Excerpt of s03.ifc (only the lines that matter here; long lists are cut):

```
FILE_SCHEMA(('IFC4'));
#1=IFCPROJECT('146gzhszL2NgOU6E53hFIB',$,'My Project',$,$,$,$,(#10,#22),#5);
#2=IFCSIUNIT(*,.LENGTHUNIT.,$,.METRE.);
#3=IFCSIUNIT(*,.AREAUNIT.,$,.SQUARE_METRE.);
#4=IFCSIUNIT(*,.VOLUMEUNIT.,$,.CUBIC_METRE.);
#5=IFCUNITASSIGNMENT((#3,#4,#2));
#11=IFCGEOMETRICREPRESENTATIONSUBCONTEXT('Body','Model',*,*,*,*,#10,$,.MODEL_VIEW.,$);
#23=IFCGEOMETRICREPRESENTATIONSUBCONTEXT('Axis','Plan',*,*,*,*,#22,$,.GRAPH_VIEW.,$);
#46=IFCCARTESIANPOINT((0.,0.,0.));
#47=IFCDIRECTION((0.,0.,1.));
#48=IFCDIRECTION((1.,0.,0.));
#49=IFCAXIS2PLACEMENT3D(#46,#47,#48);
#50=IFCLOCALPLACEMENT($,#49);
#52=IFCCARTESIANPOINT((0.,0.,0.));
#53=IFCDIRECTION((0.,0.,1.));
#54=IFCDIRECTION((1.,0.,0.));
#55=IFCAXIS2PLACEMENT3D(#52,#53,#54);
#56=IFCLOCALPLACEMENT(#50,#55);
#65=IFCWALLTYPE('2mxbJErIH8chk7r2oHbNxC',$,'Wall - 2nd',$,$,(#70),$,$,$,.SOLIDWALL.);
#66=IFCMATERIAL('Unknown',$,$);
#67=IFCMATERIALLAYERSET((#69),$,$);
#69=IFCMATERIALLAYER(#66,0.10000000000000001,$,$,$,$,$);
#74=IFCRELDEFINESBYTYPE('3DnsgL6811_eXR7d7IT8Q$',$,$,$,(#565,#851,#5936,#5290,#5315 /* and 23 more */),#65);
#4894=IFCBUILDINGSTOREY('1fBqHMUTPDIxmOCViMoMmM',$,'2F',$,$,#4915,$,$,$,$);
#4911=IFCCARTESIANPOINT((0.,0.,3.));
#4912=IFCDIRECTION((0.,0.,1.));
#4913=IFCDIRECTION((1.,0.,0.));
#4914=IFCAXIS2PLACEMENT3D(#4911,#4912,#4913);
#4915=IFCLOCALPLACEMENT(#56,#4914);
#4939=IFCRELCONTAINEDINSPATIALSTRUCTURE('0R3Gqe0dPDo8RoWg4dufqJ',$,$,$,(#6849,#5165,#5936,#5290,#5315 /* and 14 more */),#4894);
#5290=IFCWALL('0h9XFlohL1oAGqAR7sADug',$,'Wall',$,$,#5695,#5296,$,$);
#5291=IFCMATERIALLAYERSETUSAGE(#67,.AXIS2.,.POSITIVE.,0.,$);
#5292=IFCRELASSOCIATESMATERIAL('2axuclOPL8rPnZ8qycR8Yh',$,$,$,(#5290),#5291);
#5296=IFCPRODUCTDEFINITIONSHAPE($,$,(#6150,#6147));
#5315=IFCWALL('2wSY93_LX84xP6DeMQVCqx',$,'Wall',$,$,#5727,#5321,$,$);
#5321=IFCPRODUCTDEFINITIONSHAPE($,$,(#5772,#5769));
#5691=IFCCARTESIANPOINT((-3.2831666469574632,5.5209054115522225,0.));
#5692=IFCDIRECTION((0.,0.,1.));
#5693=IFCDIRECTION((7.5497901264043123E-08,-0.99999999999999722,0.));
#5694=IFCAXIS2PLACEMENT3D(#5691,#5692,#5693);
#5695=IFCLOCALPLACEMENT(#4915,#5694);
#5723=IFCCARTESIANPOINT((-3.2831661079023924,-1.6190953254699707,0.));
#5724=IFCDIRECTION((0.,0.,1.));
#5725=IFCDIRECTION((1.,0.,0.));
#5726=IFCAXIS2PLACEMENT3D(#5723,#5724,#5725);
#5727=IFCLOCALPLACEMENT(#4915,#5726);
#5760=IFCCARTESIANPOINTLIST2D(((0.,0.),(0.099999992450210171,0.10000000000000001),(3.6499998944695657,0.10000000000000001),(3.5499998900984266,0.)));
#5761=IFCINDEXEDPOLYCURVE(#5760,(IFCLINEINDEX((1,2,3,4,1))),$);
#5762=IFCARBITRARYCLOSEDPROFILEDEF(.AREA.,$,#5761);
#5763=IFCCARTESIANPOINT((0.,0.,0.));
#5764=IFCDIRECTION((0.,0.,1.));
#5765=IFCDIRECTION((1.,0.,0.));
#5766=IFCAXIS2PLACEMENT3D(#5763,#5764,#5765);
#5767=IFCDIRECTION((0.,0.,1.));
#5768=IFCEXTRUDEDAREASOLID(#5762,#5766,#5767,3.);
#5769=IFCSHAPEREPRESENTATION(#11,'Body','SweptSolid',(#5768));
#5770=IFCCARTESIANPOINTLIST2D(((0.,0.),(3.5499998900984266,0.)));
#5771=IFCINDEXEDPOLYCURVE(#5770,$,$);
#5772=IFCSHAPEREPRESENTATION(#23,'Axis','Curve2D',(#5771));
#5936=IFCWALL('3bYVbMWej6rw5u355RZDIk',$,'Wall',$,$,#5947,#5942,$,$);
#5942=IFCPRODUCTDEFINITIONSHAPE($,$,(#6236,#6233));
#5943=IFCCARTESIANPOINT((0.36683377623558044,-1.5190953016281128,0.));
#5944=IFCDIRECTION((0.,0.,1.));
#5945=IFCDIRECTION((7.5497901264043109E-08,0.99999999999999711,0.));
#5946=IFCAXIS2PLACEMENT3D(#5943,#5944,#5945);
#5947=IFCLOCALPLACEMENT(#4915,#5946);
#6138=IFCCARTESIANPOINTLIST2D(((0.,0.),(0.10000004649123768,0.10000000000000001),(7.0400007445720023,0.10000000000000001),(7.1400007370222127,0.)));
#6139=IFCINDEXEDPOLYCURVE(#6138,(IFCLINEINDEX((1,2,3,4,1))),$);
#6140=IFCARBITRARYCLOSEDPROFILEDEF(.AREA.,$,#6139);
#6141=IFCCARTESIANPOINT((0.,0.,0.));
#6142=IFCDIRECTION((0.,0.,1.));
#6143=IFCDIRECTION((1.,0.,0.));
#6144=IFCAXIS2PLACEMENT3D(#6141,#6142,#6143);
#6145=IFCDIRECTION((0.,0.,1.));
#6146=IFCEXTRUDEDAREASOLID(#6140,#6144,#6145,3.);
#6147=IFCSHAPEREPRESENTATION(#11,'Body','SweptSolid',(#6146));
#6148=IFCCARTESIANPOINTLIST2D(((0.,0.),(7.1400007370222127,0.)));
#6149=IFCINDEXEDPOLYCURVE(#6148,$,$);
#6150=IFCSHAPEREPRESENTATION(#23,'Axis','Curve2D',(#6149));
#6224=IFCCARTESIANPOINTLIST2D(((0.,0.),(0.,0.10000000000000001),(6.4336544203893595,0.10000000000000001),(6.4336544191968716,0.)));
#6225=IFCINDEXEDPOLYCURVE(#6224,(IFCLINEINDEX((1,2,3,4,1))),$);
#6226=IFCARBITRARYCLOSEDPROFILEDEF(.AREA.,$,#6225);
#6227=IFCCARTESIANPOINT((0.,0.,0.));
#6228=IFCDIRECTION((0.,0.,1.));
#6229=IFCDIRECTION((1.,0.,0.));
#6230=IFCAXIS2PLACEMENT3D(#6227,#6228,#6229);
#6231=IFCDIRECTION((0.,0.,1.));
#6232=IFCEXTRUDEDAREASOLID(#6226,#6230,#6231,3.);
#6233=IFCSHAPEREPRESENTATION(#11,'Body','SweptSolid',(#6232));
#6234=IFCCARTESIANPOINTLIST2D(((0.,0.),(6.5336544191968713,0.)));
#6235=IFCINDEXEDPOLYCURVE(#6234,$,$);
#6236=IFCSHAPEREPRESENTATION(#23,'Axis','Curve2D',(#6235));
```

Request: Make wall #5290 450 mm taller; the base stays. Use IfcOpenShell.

```python
import ifcopenshell
import ifcopenshell.geom
import ifcopenshell.util.representation
import ifcopenshell.util.shape
import ifcopenshell.util.unit

model = ifcopenshell.open("s03.ifc")
unit_scale = ifcopenshell.util.unit.calculate_unit_scale(model)
settings = ifcopenshell.geom.settings()


def volume(element):
    """Net volume in cubic metres, openings subtracted."""
    shape = ifcopenshell.geom.create_shape(settings, element)
    return ifcopenshell.util.shape.get_volume(shape.geometry)


wall = model.by_guid("0h9XFlohL1oAGqAR7sADug")
before = volume(wall)

body = ifcopenshell.util.representation.get_representation(wall, "Model", "Body")
solid = body.Items[0]
old_height = solid.Depth
solid.Depth += 0.45 / unit_scale
after = volume(wall)

print(f"height {old_height:g} -> {solid.Depth:g}, volume {before:.3f} -> {after:.3f} m3")

model.write("s03-out.ifc")
```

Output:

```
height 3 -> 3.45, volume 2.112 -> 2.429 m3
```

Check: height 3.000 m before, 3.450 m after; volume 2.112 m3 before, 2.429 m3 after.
